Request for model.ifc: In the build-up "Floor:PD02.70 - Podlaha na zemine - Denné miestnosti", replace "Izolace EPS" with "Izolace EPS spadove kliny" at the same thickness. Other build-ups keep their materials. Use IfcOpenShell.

First a look at what the model holds.

```python
import ifcopenshell
import ifcopenshell.util.element

model = ifcopenshell.open("model.ifc")
print(model.schema)
for layer_set in model.by_type("IfcMaterialLayerSet"):
    if layer_set.LayerSetName == "Floor:PD02.70 - Podlaha na zemine - Denné miestnosti":
        for layer in layer_set.MaterialLayers:
            print(layer.id(), layer.Material and layer.Material.Name, layer.LayerThickness, sep=" | ")
        print(len(ifcopenshell.util.element.get_elements_by_material(model, layer_set)), "elements and types use it")
print(sorted(m.Name for m in model.by_type("IfcMaterial") if m.Name)[:60])
```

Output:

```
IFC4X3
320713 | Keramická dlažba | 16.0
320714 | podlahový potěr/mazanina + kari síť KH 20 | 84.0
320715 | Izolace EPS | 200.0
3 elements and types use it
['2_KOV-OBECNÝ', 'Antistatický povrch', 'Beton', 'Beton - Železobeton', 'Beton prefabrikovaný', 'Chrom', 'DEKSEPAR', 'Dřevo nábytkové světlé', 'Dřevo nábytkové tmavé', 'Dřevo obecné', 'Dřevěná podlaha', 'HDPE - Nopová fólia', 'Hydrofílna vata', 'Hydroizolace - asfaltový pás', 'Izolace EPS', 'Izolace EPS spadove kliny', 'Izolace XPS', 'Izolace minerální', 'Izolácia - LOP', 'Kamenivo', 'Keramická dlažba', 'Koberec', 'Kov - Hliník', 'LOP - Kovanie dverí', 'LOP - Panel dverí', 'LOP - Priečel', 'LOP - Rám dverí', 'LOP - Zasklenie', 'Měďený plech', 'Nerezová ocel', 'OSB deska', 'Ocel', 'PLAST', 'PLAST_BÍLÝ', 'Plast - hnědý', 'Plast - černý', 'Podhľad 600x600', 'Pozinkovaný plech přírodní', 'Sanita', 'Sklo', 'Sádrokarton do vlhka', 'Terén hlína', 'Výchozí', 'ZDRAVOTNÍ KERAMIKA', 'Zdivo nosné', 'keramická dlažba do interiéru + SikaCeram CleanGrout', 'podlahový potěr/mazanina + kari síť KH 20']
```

```python
import ifcopenshell
import ifcopenshell.api.material

model = ifcopenshell.open("model.ifc")

layer_set = next(s for s in model.by_type("IfcMaterialLayerSet") if s.LayerSetName == "Floor:PD02.70 - Podlaha na zemine - Denné miestnosti")
layer = next(l for l in layer_set.MaterialLayers if l.Material and l.Material.Name == "Izolace EPS")
material = next(m for m in model.by_type("IfcMaterial") if m.Name == "Izolace EPS spadove kliny")

# Point this one layer at the other material; renaming the old one would change it everywhere.
ifcopenshell.api.material.edit_layer(model, layer=layer, attributes={"Name": material.Name}, material=material)

print([l.Material.Name if l.Material else None for l in layer_set.MaterialLayers])

model.write("model_v2.ifc")
```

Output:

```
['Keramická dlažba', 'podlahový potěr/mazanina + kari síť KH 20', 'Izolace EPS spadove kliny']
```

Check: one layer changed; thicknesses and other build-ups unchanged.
